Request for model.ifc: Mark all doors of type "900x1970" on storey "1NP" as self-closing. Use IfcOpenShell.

First a look at what the model holds.

```python
import ifcopenshell
import ifcopenshell.util.element

model = ifcopenshell.open("model.ifc")
print(model.schema)
storey = next(s for s in model.by_type("IfcBuildingStorey") if s.Name == "1NP")
doors = [e for e in ifcopenshell.util.element.get_decomposition(storey) if e.is_a("IfcDoor")]
seen = {}
for e in doors:
    element_type = ifcopenshell.util.element.get_type(e)
    key = (element_type.Name if element_type != e and element_type else None, ifcopenshell.util.element.get_pset(e, "Pset_DoorCommon", "SelfClosing"))
    seen[key] = seen.get(key, 0) + 1
for (name, value), count in sorted(seen.items(), key=str):
    print(count, "x", name, "|", value)
```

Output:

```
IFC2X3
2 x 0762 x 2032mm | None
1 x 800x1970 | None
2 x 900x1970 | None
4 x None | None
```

```python
import ifcopenshell
import ifcopenshell.api.pset
import ifcopenshell.util.element

model = ifcopenshell.open("model.ifc")

storey = next(s for s in model.by_type("IfcBuildingStorey") if s.Name == "1NP")
doors = [e for e in ifcopenshell.util.element.get_decomposition(storey) if e.is_a("IfcDoor")]

count = 0
for e in doors:
    element_type = ifcopenshell.util.element.get_type(e)
    if element_type in (None, e) or element_type.Name != "900x1970":
        continue
    # add_pset returns the element's existing set when there is one.
    pset = ifcopenshell.api.pset.add_pset(model, product=e, name="Pset_DoorCommon")
    ifcopenshell.api.pset.edit_pset(model, pset=pset, properties={"SelfClosing": True})
    count += 1

print(count, "doors updated")

model.write("model-out.ifc")
```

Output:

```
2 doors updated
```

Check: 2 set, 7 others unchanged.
